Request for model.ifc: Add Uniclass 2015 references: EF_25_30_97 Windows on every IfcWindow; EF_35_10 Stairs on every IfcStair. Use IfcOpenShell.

First a look at what the model holds.

```python
import ifcopenshell

model = ifcopenshell.open("model.ifc")
print(model.schema)
print("classifications:", [c.Name for c in model.by_type("IfcClassification")])
for ifc_class in ("IfcDoor", "IfcRoof", "IfcStair", "IfcWall", "IfcWindow"):
    print(ifc_class, len(model.by_type(ifc_class)))
```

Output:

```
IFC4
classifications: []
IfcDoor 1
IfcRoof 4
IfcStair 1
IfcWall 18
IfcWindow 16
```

```python
import ifcopenshell
import ifcopenshell.api.classification

model = ifcopenshell.open("model.ifc")

system = ifcopenshell.api.classification.add_classification(model, classification="Uniclass 2015")

codes = {
    "IfcWindow": ("EF_25_30_97", "Windows"),
    "IfcStair": ("EF_35_10", "Stairs"),
}
for ifc_class, (code, name) in codes.items():
    products = model.by_type(ifc_class)
    ifcopenshell.api.classification.add_reference(
        model, products=products, classification=system, identification=code, name=name
    )
    print(code, len(products))

model.write("model_rev.ifc")
```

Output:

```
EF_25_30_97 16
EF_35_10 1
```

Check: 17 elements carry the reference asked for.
